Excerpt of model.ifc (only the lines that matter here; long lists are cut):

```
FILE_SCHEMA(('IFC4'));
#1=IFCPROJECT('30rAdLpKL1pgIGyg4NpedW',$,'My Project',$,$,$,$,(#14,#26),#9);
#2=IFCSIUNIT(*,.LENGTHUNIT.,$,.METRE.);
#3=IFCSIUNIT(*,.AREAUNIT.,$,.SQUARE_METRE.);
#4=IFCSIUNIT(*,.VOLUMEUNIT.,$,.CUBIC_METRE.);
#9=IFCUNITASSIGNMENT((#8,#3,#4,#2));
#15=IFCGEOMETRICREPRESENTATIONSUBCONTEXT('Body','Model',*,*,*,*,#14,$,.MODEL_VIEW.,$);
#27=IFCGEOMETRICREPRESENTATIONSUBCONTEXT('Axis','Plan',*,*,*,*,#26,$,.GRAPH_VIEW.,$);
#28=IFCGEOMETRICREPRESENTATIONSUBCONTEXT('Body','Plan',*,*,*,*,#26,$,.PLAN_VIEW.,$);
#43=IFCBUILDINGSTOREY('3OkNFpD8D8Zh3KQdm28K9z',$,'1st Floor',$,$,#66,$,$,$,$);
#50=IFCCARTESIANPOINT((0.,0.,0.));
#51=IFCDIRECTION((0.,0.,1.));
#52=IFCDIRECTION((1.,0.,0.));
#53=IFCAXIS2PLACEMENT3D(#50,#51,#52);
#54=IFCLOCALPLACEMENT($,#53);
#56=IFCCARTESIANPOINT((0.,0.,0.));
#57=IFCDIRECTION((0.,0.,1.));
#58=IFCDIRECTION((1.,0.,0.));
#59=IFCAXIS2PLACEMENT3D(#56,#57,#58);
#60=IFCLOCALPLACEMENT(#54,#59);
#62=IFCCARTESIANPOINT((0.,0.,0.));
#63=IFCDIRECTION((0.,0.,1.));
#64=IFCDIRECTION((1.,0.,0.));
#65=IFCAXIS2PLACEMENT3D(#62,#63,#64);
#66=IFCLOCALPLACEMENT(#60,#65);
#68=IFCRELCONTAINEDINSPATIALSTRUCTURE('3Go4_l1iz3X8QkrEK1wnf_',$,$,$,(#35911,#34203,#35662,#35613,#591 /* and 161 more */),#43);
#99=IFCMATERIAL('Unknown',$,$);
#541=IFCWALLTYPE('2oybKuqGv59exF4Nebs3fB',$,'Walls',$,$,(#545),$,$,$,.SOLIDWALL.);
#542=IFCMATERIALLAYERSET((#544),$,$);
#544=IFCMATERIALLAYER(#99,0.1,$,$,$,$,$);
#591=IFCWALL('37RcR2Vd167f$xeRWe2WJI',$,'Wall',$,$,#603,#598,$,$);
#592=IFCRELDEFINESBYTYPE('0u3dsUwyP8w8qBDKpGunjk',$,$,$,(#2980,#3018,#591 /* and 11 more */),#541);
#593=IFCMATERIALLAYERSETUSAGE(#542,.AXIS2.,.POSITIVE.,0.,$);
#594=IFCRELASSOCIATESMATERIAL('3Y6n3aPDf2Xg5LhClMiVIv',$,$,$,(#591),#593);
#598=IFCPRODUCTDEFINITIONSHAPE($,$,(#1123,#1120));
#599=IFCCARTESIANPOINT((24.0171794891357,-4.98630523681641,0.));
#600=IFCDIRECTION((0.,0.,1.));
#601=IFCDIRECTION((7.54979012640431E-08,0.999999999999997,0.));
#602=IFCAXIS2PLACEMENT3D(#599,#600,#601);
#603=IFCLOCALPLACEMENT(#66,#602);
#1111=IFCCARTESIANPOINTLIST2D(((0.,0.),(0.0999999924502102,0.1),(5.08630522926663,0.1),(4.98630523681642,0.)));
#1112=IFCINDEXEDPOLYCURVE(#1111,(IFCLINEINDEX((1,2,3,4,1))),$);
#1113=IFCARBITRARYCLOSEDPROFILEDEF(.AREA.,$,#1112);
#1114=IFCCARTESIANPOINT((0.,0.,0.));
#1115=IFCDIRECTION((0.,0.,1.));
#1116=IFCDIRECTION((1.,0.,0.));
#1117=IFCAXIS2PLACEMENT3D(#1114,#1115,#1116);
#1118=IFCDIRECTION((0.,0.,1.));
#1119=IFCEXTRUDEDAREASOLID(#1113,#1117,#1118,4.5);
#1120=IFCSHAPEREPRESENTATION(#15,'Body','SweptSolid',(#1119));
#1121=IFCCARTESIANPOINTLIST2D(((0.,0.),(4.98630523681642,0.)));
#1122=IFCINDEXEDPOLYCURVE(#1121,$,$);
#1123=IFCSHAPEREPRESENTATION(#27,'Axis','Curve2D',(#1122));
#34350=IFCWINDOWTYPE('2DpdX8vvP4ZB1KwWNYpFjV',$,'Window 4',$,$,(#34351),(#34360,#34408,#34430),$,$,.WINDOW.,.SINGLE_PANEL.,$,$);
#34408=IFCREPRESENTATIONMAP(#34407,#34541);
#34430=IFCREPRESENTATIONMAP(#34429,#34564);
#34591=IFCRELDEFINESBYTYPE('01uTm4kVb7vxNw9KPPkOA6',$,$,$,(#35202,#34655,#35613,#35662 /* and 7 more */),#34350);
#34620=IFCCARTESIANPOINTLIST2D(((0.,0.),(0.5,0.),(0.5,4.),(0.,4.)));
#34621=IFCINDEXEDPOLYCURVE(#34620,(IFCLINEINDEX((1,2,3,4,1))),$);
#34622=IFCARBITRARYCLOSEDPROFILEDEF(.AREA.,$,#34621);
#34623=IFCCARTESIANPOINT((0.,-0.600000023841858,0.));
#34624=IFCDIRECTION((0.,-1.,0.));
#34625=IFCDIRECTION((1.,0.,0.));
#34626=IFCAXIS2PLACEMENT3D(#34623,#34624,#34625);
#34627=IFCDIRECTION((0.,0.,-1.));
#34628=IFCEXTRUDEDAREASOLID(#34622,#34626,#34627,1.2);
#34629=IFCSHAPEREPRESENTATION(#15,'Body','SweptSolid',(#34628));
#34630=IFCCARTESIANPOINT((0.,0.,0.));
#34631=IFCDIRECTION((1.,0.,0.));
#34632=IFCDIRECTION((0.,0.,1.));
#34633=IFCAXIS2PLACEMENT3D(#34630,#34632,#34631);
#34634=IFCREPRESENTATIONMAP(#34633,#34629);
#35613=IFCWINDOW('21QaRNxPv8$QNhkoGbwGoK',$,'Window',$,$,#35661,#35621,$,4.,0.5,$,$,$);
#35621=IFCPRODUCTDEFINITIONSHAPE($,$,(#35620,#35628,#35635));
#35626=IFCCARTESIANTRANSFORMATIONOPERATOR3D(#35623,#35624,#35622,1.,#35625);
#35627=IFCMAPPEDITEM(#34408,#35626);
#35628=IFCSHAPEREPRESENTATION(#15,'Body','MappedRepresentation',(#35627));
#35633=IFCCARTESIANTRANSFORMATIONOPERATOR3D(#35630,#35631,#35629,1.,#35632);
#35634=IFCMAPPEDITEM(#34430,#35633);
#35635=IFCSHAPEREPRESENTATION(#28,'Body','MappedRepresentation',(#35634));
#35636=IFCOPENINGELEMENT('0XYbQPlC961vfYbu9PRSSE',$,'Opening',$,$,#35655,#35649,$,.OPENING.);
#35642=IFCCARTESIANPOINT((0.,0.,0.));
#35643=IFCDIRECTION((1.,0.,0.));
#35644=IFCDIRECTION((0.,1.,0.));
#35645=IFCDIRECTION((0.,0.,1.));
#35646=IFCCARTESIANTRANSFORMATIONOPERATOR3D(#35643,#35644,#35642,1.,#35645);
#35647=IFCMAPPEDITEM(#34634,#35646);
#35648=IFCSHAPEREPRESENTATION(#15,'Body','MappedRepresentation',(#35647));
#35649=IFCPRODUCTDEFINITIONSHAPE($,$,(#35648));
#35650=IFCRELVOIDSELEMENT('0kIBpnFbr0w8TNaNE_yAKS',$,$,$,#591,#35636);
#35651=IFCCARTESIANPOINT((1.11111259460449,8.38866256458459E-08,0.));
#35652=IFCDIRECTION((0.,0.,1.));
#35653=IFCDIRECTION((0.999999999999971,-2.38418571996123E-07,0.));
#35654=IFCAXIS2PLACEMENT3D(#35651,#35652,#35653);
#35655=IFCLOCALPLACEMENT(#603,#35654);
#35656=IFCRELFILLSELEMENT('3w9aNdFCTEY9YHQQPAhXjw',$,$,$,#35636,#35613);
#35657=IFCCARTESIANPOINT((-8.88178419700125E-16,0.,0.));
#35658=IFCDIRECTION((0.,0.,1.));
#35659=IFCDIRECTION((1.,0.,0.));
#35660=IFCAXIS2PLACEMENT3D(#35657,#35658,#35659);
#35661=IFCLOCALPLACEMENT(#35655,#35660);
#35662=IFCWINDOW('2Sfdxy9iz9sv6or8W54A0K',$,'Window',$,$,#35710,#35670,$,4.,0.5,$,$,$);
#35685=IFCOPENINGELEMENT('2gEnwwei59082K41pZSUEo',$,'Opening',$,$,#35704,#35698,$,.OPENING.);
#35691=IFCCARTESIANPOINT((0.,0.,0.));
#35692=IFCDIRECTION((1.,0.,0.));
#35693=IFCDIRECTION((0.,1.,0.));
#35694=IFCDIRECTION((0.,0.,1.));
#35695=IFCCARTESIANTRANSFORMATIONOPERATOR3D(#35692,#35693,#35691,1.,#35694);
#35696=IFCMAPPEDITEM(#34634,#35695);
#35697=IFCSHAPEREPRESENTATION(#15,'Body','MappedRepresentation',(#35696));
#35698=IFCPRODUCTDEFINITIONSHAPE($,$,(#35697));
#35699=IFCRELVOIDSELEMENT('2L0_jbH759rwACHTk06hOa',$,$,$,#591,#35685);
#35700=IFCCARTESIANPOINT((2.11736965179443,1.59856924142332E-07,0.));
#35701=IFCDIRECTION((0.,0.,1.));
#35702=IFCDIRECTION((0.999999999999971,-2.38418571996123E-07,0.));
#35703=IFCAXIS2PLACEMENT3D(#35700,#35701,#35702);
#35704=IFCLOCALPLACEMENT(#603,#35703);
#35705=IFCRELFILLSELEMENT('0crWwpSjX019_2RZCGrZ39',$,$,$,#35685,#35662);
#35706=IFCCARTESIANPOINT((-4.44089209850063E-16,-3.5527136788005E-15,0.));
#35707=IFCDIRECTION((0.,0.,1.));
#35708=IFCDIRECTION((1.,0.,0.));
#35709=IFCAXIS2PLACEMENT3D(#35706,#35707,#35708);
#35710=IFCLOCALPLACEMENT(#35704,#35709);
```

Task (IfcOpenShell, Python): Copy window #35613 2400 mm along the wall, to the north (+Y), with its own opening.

```python
import ifcopenshell
import ifcopenshell.api.feature
import ifcopenshell.api.geometry
import ifcopenshell.api.root
import ifcopenshell.geom
import ifcopenshell.util.element
import ifcopenshell.util.placement
import ifcopenshell.util.shape

model = ifcopenshell.open("model.ifc")
settings = ifcopenshell.geom.settings()


def volume(element):
    """Net volume in cubic metres, openings subtracted."""
    shape = ifcopenshell.geom.create_shape(settings, element)
    return ifcopenshell.util.shape.get_volume(shape.geometry)


window = model.by_guid("21QaRNxPv8$QNhkoGbwGoK")
opening = window.FillsVoids[0].RelatingOpeningElement
wall = opening.VoidsElements[0].RelatingBuildingElement
before = volume(wall)
shift = ifcopenshell.util.placement.get_local_placement(wall.ObjectPlacement)[:3, 0] * 2.4

# copy_class copies the void relationship, type, container and properties, but no geometry.
new_opening = ifcopenshell.api.root.copy_class(model, product=opening)
new_opening.Representation = ifcopenshell.util.element.copy_deep(
    model, opening.Representation, exclude=["IfcGeometricRepresentationContext", "IfcRepresentationMap"]
)
new_window = ifcopenshell.api.root.copy_class(model, product=window)
new_window.Representation = ifcopenshell.util.element.copy_deep(
    model, window.Representation, exclude=["IfcGeometricRepresentationContext", "IfcRepresentationMap"]
)
ifcopenshell.api.feature.add_filling(model, opening=new_opening, element=new_window)

for old, new in ((opening, new_opening), (window, new_window)):
    matrix = ifcopenshell.util.placement.get_local_placement(old.ObjectPlacement)
    matrix[:3, 3] += shift
    ifcopenshell.api.geometry.edit_object_placement(model, product=new, matrix=matrix, is_si=False)

after = volume(wall)

print(f"wall volume {before:.3f} -> {after:.3f} m3")

model.write("model-out.ifc")
```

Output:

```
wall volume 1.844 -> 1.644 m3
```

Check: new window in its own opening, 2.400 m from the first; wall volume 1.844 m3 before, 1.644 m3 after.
